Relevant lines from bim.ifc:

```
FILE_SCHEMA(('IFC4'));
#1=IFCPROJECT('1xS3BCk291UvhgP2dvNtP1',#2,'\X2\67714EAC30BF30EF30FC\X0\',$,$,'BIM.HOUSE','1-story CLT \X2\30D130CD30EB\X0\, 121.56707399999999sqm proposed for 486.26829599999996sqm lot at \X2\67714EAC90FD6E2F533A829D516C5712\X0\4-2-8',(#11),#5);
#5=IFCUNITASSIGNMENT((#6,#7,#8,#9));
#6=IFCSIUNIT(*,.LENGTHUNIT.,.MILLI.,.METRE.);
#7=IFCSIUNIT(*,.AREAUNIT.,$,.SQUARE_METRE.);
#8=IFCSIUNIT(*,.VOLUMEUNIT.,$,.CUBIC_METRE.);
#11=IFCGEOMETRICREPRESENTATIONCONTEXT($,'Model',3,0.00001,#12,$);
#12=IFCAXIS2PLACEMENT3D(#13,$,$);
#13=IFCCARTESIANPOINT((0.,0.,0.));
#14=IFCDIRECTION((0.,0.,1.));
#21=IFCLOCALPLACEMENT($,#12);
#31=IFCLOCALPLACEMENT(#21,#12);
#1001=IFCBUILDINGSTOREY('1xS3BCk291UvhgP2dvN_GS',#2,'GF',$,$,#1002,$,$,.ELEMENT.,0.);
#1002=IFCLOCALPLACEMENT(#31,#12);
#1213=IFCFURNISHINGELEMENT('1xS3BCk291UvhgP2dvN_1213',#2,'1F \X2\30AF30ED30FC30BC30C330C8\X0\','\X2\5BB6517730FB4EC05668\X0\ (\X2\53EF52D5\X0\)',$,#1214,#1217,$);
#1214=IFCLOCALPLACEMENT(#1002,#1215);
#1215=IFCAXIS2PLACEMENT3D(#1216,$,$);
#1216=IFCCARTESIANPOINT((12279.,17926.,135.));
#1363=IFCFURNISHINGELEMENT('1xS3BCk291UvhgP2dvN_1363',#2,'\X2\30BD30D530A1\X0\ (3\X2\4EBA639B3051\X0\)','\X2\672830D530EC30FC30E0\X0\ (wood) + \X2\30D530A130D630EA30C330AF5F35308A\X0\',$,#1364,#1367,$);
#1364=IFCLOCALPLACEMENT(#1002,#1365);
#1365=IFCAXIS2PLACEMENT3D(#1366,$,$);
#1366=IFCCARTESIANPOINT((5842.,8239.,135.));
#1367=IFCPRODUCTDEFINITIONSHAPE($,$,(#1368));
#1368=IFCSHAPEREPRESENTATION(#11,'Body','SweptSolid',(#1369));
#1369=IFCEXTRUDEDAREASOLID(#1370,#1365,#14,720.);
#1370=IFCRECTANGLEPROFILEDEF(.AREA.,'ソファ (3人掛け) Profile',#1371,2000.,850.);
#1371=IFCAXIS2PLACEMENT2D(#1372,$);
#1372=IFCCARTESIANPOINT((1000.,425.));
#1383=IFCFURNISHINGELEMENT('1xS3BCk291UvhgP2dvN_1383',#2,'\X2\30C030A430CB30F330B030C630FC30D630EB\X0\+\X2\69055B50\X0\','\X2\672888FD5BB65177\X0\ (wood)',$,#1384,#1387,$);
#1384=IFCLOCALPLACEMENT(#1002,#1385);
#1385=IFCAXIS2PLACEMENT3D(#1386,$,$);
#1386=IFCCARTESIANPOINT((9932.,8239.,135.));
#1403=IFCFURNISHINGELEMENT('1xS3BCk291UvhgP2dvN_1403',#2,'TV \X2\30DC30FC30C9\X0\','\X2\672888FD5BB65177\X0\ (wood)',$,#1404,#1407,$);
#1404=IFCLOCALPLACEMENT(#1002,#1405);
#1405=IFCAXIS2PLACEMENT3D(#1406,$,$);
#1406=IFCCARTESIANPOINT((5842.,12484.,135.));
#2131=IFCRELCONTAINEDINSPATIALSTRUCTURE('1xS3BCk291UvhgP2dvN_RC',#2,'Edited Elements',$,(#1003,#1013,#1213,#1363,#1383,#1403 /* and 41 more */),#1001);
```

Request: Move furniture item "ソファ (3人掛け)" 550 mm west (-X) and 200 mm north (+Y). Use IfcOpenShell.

```python
import ifcopenshell
import ifcopenshell.api.geometry
import ifcopenshell.util.placement
import ifcopenshell.util.unit

model = ifcopenshell.open("bim.ifc")
unit_scale = ifcopenshell.util.unit.calculate_unit_scale(model)

item = model.by_guid("1xS3BCk291UvhgP2dvN_1363")
matrix = ifcopenshell.util.placement.get_local_placement(item.ObjectPlacement)
matrix[0, 3] -= 0.55 / unit_scale
matrix[1, 3] += 0.2 / unit_scale
ifcopenshell.api.geometry.edit_object_placement(model, product=item, matrix=matrix, is_si=False)

print(ifcopenshell.util.placement.get_local_placement(item.ObjectPlacement).round(3) + 0.0)

model.write("bim_rev.ifc")
```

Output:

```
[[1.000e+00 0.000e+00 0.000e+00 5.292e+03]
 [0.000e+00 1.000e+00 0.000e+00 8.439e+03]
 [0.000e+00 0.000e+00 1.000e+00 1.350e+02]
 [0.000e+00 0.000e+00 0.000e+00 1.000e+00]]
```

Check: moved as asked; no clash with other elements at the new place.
